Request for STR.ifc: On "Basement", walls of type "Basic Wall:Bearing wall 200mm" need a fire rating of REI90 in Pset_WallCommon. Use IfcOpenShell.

First a look at what the model holds.

```python
import ifcopenshell
import ifcopenshell.util.element

model = ifcopenshell.open("STR.ifc")
print(model.schema)
storey = next(s for s in model.by_type("IfcBuildingStorey") if s.Name == "Basement")
walls = [e for e in ifcopenshell.util.element.get_decomposition(storey) if e.is_a("IfcWall")]
seen = {}
for e in walls:
    element_type = ifcopenshell.util.element.get_type(e)
    key = (element_type.Name if element_type != e and element_type else None, ifcopenshell.util.element.get_pset(e, "Pset_WallCommon", "FireRating"))
    seen[key] = seen.get(key, 0) + 1
for (name, value), count in sorted(seen.items(), key=str):
    print(count, "x", name, "|", value)
```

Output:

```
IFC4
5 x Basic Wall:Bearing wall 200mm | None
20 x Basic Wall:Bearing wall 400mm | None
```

```python
import ifcopenshell
import ifcopenshell.api.pset
import ifcopenshell.util.element

model = ifcopenshell.open("STR.ifc")

storey = next(s for s in model.by_type("IfcBuildingStorey") if s.Name == "Basement")
walls = [e for e in ifcopenshell.util.element.get_decomposition(storey) if e.is_a("IfcWall")]

count = 0
for e in walls:
    element_type = ifcopenshell.util.element.get_type(e)
    if element_type in (None, e) or element_type.Name != "Basic Wall:Bearing wall 200mm":
        continue
    # add_pset returns the element's existing set when there is one.
    pset = ifcopenshell.api.pset.add_pset(model, product=e, name="Pset_WallCommon")
    ifcopenshell.api.pset.edit_pset(model, pset=pset, properties={"FireRating": "REI90"})
    count += 1

print(count, "walls updated")

model.write("STR_v2.ifc")
```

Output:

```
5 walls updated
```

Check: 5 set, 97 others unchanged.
